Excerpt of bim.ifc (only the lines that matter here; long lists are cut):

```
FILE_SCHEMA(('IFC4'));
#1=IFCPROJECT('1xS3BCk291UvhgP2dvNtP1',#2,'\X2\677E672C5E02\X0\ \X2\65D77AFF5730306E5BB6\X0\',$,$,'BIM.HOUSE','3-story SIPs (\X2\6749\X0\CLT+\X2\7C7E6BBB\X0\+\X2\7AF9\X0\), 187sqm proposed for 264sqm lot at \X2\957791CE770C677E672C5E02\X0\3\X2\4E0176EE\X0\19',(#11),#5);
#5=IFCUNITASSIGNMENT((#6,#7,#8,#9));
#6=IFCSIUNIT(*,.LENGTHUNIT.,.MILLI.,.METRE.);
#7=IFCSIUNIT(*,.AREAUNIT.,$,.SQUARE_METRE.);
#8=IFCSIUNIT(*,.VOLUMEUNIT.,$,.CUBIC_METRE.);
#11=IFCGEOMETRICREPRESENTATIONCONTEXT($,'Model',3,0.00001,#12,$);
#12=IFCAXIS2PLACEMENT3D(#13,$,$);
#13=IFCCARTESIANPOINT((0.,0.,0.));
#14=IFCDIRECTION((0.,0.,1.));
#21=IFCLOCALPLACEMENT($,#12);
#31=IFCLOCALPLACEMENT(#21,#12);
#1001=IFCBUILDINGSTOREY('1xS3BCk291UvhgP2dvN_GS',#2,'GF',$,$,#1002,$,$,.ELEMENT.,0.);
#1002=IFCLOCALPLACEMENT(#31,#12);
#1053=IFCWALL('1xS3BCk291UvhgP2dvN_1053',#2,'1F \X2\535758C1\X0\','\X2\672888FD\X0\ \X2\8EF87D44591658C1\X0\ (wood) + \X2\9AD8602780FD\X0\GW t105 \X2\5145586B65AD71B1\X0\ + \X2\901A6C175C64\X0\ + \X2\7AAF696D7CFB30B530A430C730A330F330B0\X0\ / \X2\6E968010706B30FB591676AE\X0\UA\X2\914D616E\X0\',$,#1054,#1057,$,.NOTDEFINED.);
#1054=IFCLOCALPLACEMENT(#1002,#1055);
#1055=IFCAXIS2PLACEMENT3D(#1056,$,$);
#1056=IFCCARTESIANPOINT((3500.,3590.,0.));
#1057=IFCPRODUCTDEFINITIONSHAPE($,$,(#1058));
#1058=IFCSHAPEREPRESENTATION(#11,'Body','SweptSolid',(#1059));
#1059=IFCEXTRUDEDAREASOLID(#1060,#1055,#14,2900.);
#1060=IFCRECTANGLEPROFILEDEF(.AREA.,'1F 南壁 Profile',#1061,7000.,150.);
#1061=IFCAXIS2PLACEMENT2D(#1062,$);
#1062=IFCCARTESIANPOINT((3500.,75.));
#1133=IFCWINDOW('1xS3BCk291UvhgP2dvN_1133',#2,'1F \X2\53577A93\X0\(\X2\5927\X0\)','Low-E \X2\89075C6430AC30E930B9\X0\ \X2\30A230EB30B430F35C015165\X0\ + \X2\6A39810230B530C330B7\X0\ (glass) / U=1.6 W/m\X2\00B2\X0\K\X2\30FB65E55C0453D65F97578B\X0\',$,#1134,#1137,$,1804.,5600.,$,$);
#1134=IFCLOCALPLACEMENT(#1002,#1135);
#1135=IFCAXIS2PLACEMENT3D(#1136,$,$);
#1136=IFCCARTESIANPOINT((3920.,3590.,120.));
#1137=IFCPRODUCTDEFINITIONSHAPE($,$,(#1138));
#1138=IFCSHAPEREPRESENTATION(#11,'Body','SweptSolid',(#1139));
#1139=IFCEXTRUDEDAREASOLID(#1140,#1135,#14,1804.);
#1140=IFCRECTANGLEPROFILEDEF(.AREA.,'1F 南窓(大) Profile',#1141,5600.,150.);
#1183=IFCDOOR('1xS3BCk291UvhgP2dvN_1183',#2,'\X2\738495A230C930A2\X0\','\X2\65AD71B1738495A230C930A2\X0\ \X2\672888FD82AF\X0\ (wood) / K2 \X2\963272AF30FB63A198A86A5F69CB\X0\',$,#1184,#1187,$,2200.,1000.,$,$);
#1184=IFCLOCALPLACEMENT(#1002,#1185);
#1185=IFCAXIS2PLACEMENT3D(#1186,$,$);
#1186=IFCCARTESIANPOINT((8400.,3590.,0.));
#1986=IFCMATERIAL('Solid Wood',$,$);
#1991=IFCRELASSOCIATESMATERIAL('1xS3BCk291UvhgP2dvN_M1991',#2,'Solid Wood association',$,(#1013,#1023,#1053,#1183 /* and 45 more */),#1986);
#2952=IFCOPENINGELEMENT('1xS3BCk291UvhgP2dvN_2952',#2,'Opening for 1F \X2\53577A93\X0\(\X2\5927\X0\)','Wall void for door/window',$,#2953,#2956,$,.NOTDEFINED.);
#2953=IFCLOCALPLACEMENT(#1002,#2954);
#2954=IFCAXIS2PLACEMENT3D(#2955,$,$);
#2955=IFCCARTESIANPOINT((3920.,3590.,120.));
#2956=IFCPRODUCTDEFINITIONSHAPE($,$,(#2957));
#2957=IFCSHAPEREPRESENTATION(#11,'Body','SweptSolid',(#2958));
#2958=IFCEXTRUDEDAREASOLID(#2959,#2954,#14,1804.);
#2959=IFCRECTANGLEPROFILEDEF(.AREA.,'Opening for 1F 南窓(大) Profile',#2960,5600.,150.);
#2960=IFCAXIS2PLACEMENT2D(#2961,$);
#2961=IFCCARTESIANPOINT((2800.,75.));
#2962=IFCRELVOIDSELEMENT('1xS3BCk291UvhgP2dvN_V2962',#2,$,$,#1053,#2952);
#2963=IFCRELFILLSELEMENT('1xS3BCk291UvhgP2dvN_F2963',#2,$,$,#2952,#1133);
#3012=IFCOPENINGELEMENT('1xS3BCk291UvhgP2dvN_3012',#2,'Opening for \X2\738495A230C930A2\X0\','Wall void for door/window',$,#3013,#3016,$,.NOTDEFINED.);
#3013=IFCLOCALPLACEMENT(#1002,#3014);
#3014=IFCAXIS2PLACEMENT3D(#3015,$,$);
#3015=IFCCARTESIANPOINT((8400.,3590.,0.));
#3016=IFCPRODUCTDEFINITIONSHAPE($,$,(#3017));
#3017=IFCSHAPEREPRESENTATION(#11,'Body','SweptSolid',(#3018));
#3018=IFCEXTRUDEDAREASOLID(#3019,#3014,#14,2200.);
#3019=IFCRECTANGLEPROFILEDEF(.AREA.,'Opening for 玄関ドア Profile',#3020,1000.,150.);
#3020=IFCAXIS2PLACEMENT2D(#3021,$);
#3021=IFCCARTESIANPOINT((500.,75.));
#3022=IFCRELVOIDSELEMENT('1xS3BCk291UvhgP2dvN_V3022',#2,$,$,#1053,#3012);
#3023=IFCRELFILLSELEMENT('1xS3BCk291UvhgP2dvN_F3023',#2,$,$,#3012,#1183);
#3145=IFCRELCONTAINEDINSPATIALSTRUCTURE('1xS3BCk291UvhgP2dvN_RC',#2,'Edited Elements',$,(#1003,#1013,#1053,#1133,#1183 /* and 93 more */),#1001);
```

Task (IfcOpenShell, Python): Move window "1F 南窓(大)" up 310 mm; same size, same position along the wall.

```python
import numpy as np
import ifcopenshell
import ifcopenshell.api.geometry
import ifcopenshell.util.placement
import ifcopenshell.util.unit

model = ifcopenshell.open("bim.ifc")
unit_scale = ifcopenshell.util.unit.calculate_unit_scale(model)

window = model.by_guid("1xS3BCk291UvhgP2dvN_1133")
opening = window.FillsVoids[0].RelatingOpeningElement
dz = 0.31 / unit_scale

shift = np.array([0.0, 0.0, dz])
# The window is not placed relative to its opening, so move both.
for product in (opening, window):
    matrix = ifcopenshell.util.placement.get_local_placement(product.ObjectPlacement)
    matrix[:3, 3] += shift
    ifcopenshell.api.geometry.edit_object_placement(model, product=product, matrix=matrix, is_si=False)

print(f"moved by {dz * unit_scale:+.3f} m")

model.write("bim_v2.ifc")
```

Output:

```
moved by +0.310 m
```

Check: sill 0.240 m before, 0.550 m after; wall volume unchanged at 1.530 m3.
